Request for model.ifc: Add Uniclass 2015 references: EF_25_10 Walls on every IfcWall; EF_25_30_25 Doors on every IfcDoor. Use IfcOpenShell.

First a look at what the model holds.

```python
import ifcopenshell

model = ifcopenshell.open("model.ifc")
print(model.schema)
print("classifications:", [c.Name for c in model.by_type("IfcClassification")])
for ifc_class in ("IfcDoor", "IfcRoof", "IfcStair", "IfcWall", "IfcWindow"):
    print(ifc_class, len(model.by_type(ifc_class)))
```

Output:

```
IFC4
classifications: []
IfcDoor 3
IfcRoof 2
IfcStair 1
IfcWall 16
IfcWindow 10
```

```python
import ifcopenshell
import ifcopenshell.api.classification

model = ifcopenshell.open("model.ifc")

system = ifcopenshell.api.classification.add_classification(model, classification="Uniclass 2015")

codes = {
    "IfcWall": ("EF_25_10", "Walls"),
    "IfcDoor": ("EF_25_30_25", "Doors"),
}
for ifc_class, (code, name) in codes.items():
    products = model.by_type(ifc_class)
    ifcopenshell.api.classification.add_reference(
        model, products=products, classification=system, identification=code, name=name
    )
    print(code, len(products))

model.write("model_edited.ifc")
```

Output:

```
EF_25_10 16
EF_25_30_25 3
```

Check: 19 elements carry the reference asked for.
